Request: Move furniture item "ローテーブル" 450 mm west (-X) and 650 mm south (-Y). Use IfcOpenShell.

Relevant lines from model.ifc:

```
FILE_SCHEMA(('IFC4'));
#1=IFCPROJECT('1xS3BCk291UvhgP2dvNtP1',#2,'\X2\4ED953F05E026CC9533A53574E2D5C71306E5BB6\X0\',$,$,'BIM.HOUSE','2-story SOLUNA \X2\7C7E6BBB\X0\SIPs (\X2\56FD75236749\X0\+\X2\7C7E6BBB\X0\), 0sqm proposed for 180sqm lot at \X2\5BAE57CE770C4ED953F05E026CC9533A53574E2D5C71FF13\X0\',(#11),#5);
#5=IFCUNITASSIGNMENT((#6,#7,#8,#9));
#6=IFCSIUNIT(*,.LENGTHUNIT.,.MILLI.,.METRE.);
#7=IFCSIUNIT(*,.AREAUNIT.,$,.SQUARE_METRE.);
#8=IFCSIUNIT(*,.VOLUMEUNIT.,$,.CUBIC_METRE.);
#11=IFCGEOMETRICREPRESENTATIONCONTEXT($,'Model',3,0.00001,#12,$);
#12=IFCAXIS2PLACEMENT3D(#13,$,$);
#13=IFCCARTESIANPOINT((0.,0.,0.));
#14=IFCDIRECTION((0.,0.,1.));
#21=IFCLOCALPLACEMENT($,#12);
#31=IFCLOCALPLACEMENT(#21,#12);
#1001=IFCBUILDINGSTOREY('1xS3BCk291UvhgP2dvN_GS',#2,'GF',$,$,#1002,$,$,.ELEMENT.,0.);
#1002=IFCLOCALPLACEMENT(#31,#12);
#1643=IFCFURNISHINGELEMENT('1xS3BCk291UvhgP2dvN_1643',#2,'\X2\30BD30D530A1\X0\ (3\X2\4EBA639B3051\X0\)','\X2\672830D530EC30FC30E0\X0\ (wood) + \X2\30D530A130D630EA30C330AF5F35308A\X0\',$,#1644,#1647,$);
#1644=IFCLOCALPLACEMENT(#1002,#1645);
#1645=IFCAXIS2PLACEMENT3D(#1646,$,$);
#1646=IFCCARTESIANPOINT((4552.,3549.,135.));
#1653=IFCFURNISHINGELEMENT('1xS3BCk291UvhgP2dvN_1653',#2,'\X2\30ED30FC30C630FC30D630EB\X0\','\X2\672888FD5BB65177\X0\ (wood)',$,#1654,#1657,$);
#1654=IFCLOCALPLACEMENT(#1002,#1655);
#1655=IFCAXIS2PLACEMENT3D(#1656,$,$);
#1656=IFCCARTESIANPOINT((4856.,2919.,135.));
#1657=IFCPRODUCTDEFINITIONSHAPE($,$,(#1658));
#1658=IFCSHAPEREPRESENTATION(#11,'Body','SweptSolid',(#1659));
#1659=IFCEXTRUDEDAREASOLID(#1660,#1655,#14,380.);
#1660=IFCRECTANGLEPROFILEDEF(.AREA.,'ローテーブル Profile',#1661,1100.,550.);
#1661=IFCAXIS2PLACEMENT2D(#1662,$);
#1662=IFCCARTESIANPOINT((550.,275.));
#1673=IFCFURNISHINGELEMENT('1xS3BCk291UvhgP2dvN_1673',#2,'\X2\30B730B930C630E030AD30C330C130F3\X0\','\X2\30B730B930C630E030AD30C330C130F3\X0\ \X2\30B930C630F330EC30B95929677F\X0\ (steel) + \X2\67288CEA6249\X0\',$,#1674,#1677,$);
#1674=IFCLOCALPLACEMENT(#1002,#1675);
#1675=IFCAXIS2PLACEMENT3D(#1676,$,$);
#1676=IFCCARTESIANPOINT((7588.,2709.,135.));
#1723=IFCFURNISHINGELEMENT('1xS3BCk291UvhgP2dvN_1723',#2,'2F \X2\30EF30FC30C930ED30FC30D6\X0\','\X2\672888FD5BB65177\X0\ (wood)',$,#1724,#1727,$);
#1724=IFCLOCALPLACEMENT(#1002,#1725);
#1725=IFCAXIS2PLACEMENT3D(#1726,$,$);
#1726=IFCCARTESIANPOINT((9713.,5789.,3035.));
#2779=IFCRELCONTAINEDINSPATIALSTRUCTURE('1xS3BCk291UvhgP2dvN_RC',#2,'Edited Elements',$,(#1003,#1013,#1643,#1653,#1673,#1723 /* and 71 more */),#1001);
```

```python
import ifcopenshell
import ifcopenshell.api.geometry
import ifcopenshell.util.placement

model = ifcopenshell.open("model.ifc")

item = model.by_guid("1xS3BCk291UvhgP2dvN_1653")
matrix = ifcopenshell.util.placement.get_local_placement(item.ObjectPlacement)
matrix[0, 3] -= 450.0
matrix[1, 3] -= 650.0
ifcopenshell.api.geometry.edit_object_placement(model, product=item, matrix=matrix, is_si=False)

print(ifcopenshell.util.placement.get_local_placement(item.ObjectPlacement).round(3) + 0.0)

model.write("model-out.ifc")
```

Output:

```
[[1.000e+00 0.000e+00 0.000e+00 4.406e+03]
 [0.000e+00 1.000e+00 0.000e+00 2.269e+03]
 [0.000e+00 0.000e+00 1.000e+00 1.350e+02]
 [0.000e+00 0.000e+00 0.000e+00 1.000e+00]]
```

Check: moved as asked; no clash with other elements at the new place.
